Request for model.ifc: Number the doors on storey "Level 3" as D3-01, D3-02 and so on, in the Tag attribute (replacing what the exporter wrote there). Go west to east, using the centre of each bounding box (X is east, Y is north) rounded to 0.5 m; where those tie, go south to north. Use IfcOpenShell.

First a look at what the model holds.

```python
import ifcopenshell
import ifcopenshell.util.element
import ifcopenshell.util.placement

model = ifcopenshell.open("model.ifc")
print(model.schema)
storey = next(s for s in model.by_type("IfcBuildingStorey") if s.Name == "Level 3")
doors = [e for e in ifcopenshell.util.element.get_decomposition(storey) if e.is_a("IfcDoor")]
for e in sorted(doors, key=lambda e: e.id()):
    origin = ifcopenshell.util.placement.get_local_placement(e.ObjectPlacement)[:3, 3]
    print(e.id(), e.Tag, e.Name, origin.round(2) + 0.0, sep=" | ")
```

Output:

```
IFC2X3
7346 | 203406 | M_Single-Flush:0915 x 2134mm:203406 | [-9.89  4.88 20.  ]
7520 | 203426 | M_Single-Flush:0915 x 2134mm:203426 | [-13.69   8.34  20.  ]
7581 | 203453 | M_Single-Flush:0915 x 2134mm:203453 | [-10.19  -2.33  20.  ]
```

```python
import ifcopenshell
import ifcopenshell.geom
import ifcopenshell.util.element
import ifcopenshell.util.shape

model = ifcopenshell.open("model.ifc")
settings = ifcopenshell.geom.settings()
settings.set("use-world-coords", True)


def centre(element):
    shape = ifcopenshell.geom.create_shape(settings, element)
    return ifcopenshell.util.shape.get_bbox_centroid(shape.geometry)


storey = next(s for s in model.by_type("IfcBuildingStorey") if s.Name == "Level 3")
doors = [e for e in ifcopenshell.util.element.get_decomposition(storey) if e.is_a("IfcDoor")]

# Insertion points can sit at a corner or the storey origin, so sort by the geometry (in metres).
centres = {e: centre(e) for e in doors}
doors.sort(key=lambda e: (round(centres[e][0] / 0.5), centres[e][1]))

for i, e in enumerate(doors, start=1):
    number = f"D3-{i:02d}"
    e.Tag = number
    print(e.id(), number)

model.write("model_edited.ifc")
```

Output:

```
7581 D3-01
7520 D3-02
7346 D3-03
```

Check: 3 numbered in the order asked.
